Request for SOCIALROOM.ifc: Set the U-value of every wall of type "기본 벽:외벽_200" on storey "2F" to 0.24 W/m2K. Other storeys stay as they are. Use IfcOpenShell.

First a look at what the model holds.

```python
import ifcopenshell
import ifcopenshell.util.element

model = ifcopenshell.open("SOCIALROOM.ifc")
print(model.schema)
storey = next(s for s in model.by_type("IfcBuildingStorey") if s.Name == "2F")
walls = [e for e in ifcopenshell.util.element.get_decomposition(storey) if e.is_a("IfcWall")]
seen = {}
for e in walls:
    element_type = ifcopenshell.util.element.get_type(e)
    key = (element_type.Name if element_type != e and element_type else None, ifcopenshell.util.element.get_pset(e, "Pset_WallCommon", "ThermalTransmittance"))
    seen[key] = seen.get(key, 0) + 1
for (name, value), count in sorted(seen.items(), key=str):
    print(count, "x", name, "|", value)
```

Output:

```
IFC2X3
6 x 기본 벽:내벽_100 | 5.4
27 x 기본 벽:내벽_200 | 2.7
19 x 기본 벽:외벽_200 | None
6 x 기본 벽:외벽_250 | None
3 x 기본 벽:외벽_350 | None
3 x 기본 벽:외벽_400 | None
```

```python
import ifcopenshell
import ifcopenshell.api.pset
import ifcopenshell.util.element

model = ifcopenshell.open("SOCIALROOM.ifc")

storey = next(s for s in model.by_type("IfcBuildingStorey") if s.Name == "2F")
walls = [e for e in ifcopenshell.util.element.get_decomposition(storey) if e.is_a("IfcWall")]

count = 0
for e in walls:
    element_type = ifcopenshell.util.element.get_type(e)
    if element_type in (None, e) or element_type.Name != "기본 벽:외벽_200":
        continue
    # add_pset returns the element's existing set when there is one.
    pset = ifcopenshell.api.pset.add_pset(model, product=e, name="Pset_WallCommon")
    ifcopenshell.api.pset.edit_pset(model, pset=pset, properties={"ThermalTransmittance": 0.24})
    count += 1

print(count, "walls updated")

model.write("SOCIALROOM-out.ifc")
```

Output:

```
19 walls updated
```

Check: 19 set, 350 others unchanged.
